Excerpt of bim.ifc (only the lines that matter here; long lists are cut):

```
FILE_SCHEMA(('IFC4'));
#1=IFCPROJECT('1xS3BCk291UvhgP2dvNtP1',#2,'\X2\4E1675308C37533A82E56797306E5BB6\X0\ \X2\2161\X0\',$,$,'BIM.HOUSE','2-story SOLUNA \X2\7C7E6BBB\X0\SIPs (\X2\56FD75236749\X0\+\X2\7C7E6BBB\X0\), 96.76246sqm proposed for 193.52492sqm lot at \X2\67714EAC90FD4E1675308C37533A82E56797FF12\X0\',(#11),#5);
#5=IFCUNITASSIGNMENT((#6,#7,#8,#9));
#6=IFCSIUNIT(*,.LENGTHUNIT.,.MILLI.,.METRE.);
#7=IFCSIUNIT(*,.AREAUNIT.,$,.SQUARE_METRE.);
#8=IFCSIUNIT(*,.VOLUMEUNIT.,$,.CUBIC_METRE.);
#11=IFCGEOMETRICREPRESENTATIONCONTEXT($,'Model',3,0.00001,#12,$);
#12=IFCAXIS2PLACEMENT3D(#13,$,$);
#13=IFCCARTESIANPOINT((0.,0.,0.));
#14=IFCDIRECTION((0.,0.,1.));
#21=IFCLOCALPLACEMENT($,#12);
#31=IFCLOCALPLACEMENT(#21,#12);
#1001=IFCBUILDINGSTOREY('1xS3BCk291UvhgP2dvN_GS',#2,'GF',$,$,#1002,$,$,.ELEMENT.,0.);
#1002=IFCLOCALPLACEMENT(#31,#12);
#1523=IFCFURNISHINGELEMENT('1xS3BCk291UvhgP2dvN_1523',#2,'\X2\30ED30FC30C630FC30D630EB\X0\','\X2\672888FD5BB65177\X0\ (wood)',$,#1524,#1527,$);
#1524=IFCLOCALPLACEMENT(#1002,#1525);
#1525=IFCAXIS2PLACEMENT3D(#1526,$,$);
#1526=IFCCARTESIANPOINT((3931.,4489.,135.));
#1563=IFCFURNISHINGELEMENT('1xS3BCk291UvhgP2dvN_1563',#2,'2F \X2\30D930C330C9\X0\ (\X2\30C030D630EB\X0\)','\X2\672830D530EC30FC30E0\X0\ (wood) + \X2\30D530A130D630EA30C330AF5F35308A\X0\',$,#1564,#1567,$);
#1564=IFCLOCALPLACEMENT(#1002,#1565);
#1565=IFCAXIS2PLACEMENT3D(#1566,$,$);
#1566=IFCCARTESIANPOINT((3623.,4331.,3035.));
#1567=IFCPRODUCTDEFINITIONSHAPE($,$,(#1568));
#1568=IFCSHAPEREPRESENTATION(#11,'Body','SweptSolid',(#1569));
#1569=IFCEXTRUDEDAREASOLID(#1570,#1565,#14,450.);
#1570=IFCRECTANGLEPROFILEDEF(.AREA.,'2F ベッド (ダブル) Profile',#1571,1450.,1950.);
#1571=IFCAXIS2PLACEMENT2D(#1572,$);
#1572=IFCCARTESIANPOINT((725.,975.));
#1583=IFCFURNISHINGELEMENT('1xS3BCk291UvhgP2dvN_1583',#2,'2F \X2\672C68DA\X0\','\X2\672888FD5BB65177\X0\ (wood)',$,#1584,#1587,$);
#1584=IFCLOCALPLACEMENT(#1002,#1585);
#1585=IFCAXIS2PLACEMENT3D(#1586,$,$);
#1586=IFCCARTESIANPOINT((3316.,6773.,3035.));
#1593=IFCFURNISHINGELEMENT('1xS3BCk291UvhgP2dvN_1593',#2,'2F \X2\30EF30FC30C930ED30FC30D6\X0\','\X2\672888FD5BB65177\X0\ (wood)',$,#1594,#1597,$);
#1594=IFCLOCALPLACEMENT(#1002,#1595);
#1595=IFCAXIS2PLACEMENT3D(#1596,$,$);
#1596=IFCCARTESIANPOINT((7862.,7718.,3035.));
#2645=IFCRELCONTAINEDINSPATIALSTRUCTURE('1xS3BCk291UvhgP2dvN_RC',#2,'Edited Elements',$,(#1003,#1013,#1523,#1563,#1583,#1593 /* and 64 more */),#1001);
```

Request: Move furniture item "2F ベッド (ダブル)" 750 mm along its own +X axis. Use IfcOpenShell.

```python
import ifcopenshell
import ifcopenshell.api.geometry
import ifcopenshell.util.placement
import ifcopenshell.util.unit

model = ifcopenshell.open("bim.ifc")
unit_scale = ifcopenshell.util.unit.calculate_unit_scale(model)

item = model.by_guid("1xS3BCk291UvhgP2dvN_1563")
matrix = ifcopenshell.util.placement.get_local_placement(item.ObjectPlacement)
matrix[:3, 3] += matrix[:3, 0] * 0.75 / unit_scale
ifcopenshell.api.geometry.edit_object_placement(model, product=item, matrix=matrix, is_si=False)

print(ifcopenshell.util.placement.get_local_placement(item.ObjectPlacement).round(3) + 0.0)

model.write("bim-out.ifc")
```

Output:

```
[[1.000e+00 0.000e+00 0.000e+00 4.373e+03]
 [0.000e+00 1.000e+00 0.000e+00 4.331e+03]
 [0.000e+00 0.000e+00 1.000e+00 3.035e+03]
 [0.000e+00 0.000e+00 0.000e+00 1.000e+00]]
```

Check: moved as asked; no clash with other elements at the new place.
